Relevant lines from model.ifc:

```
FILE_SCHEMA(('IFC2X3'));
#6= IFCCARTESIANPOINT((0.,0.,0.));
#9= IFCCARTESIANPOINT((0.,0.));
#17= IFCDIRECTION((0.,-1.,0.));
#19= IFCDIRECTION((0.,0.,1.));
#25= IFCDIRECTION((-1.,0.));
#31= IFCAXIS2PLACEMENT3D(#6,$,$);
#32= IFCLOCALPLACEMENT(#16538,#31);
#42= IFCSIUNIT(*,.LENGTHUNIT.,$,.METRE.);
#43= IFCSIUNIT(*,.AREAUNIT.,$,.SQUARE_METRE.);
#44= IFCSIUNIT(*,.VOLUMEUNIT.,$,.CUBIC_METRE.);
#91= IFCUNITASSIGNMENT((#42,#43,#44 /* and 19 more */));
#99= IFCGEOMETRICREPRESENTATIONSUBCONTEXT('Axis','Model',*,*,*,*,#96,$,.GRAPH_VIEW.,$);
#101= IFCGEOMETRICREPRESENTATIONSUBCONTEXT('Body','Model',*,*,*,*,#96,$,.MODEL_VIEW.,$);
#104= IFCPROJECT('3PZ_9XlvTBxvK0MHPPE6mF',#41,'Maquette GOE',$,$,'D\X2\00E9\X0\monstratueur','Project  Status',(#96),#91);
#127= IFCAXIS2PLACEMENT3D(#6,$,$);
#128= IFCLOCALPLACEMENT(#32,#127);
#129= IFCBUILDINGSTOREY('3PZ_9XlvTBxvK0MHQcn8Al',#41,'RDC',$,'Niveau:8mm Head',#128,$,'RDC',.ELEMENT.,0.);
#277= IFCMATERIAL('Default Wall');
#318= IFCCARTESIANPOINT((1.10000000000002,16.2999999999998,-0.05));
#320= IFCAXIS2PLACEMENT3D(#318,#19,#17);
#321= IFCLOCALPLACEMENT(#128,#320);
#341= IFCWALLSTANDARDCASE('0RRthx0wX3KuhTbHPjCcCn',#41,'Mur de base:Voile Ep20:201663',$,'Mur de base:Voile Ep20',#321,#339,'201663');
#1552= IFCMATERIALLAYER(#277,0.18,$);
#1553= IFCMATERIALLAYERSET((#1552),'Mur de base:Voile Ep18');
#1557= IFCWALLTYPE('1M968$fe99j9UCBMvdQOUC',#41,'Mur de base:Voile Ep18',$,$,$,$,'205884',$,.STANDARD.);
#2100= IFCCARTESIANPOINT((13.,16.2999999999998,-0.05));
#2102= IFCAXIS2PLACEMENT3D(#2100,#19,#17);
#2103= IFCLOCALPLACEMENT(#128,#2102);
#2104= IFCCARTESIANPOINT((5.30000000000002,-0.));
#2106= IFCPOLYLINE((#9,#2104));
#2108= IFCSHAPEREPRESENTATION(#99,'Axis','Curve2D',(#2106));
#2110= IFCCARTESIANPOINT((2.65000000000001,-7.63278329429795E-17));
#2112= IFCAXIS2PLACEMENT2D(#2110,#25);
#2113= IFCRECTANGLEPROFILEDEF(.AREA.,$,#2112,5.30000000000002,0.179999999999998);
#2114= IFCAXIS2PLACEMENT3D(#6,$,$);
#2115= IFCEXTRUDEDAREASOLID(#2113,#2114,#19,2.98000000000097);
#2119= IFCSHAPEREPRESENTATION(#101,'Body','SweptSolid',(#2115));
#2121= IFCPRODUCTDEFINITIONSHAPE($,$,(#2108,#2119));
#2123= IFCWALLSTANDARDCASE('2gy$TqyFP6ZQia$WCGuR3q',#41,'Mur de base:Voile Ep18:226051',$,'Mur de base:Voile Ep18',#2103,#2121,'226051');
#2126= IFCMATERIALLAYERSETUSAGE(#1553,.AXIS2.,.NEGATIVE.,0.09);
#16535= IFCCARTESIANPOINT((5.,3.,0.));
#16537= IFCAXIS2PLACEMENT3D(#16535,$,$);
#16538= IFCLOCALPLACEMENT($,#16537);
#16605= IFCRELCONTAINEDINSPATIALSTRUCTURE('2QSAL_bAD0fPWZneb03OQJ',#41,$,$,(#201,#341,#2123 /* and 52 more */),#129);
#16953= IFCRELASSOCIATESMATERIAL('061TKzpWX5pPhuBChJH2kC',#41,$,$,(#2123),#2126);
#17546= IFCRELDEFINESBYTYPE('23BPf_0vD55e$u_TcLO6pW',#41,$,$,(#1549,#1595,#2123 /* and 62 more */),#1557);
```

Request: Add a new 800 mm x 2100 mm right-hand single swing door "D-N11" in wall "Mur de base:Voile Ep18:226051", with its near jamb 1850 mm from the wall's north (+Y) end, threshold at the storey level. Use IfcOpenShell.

```python
import numpy as np
import ifcopenshell
import ifcopenshell.api.feature
import ifcopenshell.api.geometry
import ifcopenshell.api.root
import ifcopenshell.api.spatial
import ifcopenshell.api.type
import ifcopenshell.geom
import ifcopenshell.util.element
import ifcopenshell.util.placement
import ifcopenshell.util.representation
import ifcopenshell.util.shape
import ifcopenshell.util.unit

model = ifcopenshell.open("model.ifc")
unit_scale = ifcopenshell.util.unit.calculate_unit_scale(model)
settings = ifcopenshell.geom.settings()


def volume(element):
    """Net volume in cubic metres, openings subtracted."""
    shape = ifcopenshell.geom.create_shape(settings, element)
    return ifcopenshell.util.shape.get_volume(shape.geometry)


wall = model.by_id(2123)
storey = ifcopenshell.util.element.get_container(wall, ifc_class="IfcBuildingStorey")
context = ifcopenshell.util.representation.get_context(model, "Model", "Body", "MODEL_VIEW")
before = volume(wall)

width, height, from_end, sill = 0.8, 2.1, 1.85, 0.0  # metres

# The wall runs along its own X axis, and the end named is its -X end.
wall_shape = ifcopenshell.geom.create_shape(settings, wall)
x, y, z = ifcopenshell.util.shape.get_vertices(wall_shape.geometry).T
start = x.min() + from_end
face, thickness = float(y.min()), float(y.max() - y.min())
wall_matrix = ifcopenshell.util.placement.get_local_placement(wall.ObjectPlacement)
level = ifcopenshell.util.placement.get_local_placement(storey.ObjectPlacement)[2, 3]


def in_wall(x, y):
    """Placement at x, y metres in the wall's axes, at sill height."""
    matrix = wall_matrix.copy()
    matrix[:, 3] = wall_matrix @ np.array([x / unit_scale, y / unit_scale, 0.0, 1.0])
    matrix[2, 3] = level + sill / unit_scale
    return matrix


# Opening: a box that overshoots both wall faces by 50 mm.
opening = ifcopenshell.api.root.create_entity(model, ifc_class="IfcOpeningElement")
box = ifcopenshell.api.geometry.add_wall_representation(
    model, context=context, length=width, height=height, thickness=thickness + 0.1
)
ifcopenshell.api.geometry.assign_representation(model, product=opening, representation=box)
ifcopenshell.api.geometry.edit_object_placement(model, product=opening, matrix=in_wall(start, face - 0.05), is_si=False)
ifcopenshell.api.feature.add_feature(model, feature=opening, element=wall)

door = ifcopenshell.api.root.create_entity(model, ifc_class="IfcDoor", name="D-N11")
door.OverallWidth, door.OverallHeight = width / unit_scale, height / unit_scale
body = ifcopenshell.api.geometry.add_door_representation(
    model,
    context=context,
    overall_width=door.OverallWidth,
    overall_height=door.OverallHeight,
    operation_type="SINGLE_SWING_RIGHT",
    lining_properties={"LiningDepth": thickness / unit_scale, "ThresholdDepth": thickness / unit_scale},
)
ifcopenshell.api.geometry.assign_representation(model, product=door, representation=body)
ifcopenshell.api.spatial.assign_container(model, products=[door], relating_structure=storey)
fills = ifcopenshell.api.feature.add_filling(model, opening=opening, element=door)
fills.OwnerHistory = door.OwnerHistory  # required in IFC2X3

# IFC2X3 keeps the operation on the door style.
style = ifcopenshell.api.root.create_entity(model, ifc_class="IfcDoorStyle", name="D-N11")
style.OperationType, style.ConstructionType = "SINGLE_SWING_RIGHT", "NOTDEFINED"
style.ParameterTakesPrecedence = style.Sizeable = False
ifcopenshell.api.type.assign_type(model, related_objects=[door], relating_type=style)

# The lining spans the wall, so the door starts at the wall face.
ifcopenshell.api.geometry.edit_object_placement(model, product=door, matrix=in_wall(start, face), is_si=False)

after = volume(wall)

print(f"wall volume {before:.3f} -> {after:.3f} m3")

model.write("model_rev.ifc")
```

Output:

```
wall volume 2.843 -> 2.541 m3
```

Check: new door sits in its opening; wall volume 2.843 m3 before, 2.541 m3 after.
